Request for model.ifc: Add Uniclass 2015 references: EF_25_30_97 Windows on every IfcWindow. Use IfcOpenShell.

First a look at what the model holds.

```python
import ifcopenshell

model = ifcopenshell.open("model.ifc")
print(model.schema)
print("classifications:", [c.Name for c in model.by_type("IfcClassification")])
for ifc_class in ("IfcDoor", "IfcRoof", "IfcStair", "IfcWall", "IfcWindow"):
    print(ifc_class, len(model.by_type(ifc_class)))
```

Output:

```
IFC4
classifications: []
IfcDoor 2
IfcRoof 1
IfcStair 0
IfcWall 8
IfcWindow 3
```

```python
import ifcopenshell
import ifcopenshell.api.classification

model = ifcopenshell.open("model.ifc")

system = ifcopenshell.api.classification.add_classification(model, classification="Uniclass 2015")

codes = {
    "IfcWindow": ("EF_25_30_97", "Windows"),
}
for ifc_class, (code, name) in codes.items():
    products = model.by_type(ifc_class)
    ifcopenshell.api.classification.add_reference(
        model, products=products, classification=system, identification=code, name=name
    )
    print(code, len(products))

model.write("model_v2.ifc")
```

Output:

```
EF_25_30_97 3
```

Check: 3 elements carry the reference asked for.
